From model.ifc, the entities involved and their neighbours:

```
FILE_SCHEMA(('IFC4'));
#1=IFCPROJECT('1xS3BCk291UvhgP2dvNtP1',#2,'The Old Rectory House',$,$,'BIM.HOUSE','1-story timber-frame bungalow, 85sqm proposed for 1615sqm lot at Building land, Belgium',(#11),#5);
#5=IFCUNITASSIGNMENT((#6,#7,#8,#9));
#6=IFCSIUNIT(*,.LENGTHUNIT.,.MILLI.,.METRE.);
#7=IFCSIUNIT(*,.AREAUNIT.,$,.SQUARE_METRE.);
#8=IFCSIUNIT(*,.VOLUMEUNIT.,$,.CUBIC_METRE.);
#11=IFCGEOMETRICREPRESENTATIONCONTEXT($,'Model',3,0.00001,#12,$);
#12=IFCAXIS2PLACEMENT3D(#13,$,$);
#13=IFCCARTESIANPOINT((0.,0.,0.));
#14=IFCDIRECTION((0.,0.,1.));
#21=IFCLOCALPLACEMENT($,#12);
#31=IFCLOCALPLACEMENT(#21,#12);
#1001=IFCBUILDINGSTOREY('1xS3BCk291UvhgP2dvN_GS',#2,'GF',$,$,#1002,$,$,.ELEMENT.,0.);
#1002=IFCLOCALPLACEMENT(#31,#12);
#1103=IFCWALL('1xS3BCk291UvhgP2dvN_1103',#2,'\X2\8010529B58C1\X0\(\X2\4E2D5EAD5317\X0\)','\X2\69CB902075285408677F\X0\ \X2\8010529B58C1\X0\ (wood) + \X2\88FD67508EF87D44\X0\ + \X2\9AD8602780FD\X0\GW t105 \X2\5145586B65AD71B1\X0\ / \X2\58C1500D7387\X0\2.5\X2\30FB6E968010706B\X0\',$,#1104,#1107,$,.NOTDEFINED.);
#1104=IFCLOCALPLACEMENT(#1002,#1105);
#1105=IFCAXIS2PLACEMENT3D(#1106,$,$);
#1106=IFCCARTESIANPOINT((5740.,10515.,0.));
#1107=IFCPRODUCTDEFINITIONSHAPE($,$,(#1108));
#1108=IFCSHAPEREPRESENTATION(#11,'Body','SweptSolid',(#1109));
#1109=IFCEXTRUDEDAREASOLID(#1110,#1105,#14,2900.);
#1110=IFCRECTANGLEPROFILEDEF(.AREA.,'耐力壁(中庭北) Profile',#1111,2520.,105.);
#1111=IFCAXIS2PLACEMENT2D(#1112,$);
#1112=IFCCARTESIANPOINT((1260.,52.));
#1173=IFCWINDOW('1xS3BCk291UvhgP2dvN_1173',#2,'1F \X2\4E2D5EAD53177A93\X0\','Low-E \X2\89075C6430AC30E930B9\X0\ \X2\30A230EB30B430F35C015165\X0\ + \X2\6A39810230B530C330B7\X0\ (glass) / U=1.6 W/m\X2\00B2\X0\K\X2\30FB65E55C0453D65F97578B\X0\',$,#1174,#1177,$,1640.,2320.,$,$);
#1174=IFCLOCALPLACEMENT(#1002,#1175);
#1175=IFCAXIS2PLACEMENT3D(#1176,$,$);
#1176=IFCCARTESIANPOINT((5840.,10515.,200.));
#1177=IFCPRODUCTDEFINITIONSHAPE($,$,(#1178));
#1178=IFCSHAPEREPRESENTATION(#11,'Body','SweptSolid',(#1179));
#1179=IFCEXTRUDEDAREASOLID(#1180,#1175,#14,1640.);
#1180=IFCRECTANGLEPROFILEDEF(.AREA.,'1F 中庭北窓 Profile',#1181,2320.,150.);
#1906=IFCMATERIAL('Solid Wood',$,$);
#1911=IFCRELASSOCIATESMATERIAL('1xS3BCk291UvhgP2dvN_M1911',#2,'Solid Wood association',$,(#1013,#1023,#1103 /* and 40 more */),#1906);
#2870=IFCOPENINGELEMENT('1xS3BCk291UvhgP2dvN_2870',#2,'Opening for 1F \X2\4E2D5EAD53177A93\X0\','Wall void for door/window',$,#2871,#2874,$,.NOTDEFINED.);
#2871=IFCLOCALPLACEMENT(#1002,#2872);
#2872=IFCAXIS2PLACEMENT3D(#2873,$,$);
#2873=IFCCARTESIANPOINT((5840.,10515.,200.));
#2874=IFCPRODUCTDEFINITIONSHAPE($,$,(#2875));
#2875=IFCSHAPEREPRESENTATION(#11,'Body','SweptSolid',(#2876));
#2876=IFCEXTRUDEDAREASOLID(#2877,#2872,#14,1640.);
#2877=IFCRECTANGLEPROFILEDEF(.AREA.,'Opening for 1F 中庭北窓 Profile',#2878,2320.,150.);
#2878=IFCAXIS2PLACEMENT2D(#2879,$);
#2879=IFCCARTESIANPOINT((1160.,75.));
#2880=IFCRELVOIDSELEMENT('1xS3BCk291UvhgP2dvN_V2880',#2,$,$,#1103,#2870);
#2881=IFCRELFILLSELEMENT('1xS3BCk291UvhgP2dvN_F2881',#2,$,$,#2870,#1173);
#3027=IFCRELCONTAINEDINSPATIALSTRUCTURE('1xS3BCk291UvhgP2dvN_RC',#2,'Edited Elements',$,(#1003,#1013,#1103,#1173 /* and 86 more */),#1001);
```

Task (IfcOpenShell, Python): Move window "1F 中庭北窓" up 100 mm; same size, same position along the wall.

```python
import numpy as np
import ifcopenshell
import ifcopenshell.api.geometry
import ifcopenshell.util.placement
import ifcopenshell.util.unit

model = ifcopenshell.open("model.ifc")
unit_scale = ifcopenshell.util.unit.calculate_unit_scale(model)

window = model.by_guid("1xS3BCk291UvhgP2dvN_1173")
opening = window.FillsVoids[0].RelatingOpeningElement
dz = 100.0

shift = np.array([0.0, 0.0, dz])
# The window is not placed relative to its opening, so move both.
for product in (opening, window):
    matrix = ifcopenshell.util.placement.get_local_placement(product.ObjectPlacement)
    matrix[:3, 3] += shift
    ifcopenshell.api.geometry.edit_object_placement(model, product=product, matrix=matrix, is_si=False)

print(f"moved by {dz * unit_scale:+.3f} m")

model.write("model_edited.ifc")
```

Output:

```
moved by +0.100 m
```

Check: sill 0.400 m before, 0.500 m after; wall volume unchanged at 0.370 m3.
